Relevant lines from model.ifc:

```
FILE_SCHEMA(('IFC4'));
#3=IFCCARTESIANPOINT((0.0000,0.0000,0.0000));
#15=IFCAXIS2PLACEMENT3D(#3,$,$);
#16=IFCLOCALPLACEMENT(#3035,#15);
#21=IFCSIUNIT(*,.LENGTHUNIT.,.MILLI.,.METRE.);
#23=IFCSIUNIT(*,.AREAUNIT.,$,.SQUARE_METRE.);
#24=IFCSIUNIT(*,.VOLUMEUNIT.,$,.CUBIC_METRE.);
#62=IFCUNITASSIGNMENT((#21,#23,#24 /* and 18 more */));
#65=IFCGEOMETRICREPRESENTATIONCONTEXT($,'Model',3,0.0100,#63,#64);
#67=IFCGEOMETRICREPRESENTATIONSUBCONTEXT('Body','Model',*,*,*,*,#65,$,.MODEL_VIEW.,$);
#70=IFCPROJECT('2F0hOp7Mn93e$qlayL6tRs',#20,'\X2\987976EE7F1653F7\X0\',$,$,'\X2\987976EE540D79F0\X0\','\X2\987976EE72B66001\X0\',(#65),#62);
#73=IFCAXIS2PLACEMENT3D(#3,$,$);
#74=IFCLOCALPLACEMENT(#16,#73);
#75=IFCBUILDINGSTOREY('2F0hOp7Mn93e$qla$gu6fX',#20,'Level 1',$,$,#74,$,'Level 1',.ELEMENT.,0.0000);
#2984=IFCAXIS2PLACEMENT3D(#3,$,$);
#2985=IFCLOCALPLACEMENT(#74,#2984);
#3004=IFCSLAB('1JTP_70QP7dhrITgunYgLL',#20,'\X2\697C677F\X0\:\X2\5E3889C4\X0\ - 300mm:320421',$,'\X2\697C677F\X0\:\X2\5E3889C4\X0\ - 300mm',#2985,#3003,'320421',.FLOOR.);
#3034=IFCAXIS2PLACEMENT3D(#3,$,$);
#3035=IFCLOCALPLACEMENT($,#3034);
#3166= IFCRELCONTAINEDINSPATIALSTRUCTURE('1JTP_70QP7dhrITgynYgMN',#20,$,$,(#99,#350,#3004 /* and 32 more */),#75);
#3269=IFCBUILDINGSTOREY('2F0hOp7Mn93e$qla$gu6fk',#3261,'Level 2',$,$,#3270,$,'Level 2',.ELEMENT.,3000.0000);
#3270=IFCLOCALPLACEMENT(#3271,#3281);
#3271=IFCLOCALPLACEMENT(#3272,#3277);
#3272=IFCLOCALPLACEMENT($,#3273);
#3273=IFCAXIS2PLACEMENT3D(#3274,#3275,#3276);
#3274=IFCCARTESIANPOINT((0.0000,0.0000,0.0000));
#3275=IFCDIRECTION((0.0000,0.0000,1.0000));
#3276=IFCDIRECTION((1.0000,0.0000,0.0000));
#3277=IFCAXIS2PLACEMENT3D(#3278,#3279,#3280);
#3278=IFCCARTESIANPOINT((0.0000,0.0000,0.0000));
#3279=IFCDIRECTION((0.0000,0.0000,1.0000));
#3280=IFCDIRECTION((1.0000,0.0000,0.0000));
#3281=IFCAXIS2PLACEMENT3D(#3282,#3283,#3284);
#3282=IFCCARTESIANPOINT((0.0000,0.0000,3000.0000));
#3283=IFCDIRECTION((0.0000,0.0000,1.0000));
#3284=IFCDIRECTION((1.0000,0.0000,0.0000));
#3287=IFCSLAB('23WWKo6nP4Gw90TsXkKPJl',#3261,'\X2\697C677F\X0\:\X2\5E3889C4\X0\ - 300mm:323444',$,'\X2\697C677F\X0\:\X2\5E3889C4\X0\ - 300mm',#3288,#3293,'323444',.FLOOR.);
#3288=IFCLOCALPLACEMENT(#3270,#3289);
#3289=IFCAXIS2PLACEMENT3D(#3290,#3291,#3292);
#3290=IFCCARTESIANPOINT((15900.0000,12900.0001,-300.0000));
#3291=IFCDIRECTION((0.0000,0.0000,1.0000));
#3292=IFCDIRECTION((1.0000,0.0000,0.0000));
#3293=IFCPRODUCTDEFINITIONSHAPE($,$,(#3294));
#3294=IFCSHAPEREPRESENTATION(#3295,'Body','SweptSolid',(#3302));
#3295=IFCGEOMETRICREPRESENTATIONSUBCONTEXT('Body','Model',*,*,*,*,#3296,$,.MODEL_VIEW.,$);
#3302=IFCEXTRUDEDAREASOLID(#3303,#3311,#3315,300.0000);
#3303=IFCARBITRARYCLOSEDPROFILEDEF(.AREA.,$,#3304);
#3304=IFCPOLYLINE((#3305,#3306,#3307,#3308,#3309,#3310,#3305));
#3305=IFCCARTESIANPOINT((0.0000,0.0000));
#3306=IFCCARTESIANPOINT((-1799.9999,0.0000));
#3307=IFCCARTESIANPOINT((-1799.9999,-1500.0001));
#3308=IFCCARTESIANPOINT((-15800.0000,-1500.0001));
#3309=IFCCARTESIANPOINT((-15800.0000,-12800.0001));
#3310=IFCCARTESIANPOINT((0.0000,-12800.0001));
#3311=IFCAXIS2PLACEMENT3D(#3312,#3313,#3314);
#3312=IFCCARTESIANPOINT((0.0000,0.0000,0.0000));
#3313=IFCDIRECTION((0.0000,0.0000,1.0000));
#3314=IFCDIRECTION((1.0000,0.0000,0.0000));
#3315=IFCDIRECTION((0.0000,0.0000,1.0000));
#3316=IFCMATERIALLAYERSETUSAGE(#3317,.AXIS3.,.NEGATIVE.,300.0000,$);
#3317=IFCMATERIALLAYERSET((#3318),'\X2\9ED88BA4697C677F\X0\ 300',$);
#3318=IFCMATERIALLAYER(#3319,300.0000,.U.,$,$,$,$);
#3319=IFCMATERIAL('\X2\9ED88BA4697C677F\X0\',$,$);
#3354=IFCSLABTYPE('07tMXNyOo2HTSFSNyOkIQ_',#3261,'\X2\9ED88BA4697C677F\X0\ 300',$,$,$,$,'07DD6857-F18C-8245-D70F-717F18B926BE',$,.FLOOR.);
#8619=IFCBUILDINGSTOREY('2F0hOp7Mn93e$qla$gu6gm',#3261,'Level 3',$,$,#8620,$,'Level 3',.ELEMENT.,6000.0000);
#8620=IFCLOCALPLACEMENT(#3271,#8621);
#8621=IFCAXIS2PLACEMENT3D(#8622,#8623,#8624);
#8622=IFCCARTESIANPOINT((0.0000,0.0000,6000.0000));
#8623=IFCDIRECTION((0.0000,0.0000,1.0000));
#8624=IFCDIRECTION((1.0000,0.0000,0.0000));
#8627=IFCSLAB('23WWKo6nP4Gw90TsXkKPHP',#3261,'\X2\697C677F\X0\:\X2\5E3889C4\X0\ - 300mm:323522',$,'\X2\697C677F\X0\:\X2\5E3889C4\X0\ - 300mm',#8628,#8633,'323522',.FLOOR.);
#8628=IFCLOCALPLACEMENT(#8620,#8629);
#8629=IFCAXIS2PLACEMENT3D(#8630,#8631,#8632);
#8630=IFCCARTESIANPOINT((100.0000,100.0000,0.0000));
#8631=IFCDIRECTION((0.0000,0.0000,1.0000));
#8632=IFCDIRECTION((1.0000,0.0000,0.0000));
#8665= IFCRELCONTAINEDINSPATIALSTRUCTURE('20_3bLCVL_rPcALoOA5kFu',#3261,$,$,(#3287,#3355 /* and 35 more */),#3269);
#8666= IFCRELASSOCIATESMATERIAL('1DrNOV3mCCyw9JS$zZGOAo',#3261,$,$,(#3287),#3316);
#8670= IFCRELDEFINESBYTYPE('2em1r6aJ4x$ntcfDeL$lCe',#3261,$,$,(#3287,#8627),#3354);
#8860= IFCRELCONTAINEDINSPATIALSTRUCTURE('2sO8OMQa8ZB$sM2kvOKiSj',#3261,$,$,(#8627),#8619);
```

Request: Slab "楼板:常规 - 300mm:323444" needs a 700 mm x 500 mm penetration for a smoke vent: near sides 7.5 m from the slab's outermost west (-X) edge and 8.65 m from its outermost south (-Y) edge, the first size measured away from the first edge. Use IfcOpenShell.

```python
import numpy as np
import ifcopenshell
import ifcopenshell.api.feature
import ifcopenshell.api.geometry
import ifcopenshell.api.root
import ifcopenshell.geom
import ifcopenshell.util.placement
import ifcopenshell.util.representation
import ifcopenshell.util.shape
import ifcopenshell.util.unit

model = ifcopenshell.open("model.ifc")
unit_scale = ifcopenshell.util.unit.calculate_unit_scale(model)
settings = ifcopenshell.geom.settings()


def volume(element):
    """Net volume in cubic metres, openings subtracted."""
    shape = ifcopenshell.geom.create_shape(settings, element)
    return ifcopenshell.util.shape.get_volume(shape.geometry)


slab = model.by_id(3287)
before = volume(slab)

# Extent in the slab's own axes, in metres. The edges named are its -X and -Y sides.
slab_shape = ifcopenshell.geom.create_shape(settings, slab)
vertices = ifcopenshell.util.shape.get_vertices(slab_shape.geometry)
x_min, y_min, bottom = vertices.min(axis=0)
top = vertices[:, 2].max()

opening = ifcopenshell.api.root.create_entity(model, ifc_class="IfcOpeningElement", name="Smoke vent opening", predefined_type="OPENING")
context = ifcopenshell.util.representation.get_context(model, "Model", "Body", "MODEL_VIEW")
width, depth = 0.7, 0.5
outline = [(0.0, 0.0), (width, 0.0), (width, depth), (0.0, depth), (0.0, 0.0)]
# Overshoot both faces by 50 mm so the cut is clean.
shape = ifcopenshell.api.geometry.add_slab_representation(
    model, context=context, depth=top - bottom + 0.1, polyline=outline
)
ifcopenshell.api.geometry.assign_representation(model, product=opening, representation=shape)

matrix = ifcopenshell.util.placement.get_local_placement(slab.ObjectPlacement)
matrix[:, 3] = matrix @ np.append(np.array([x_min + 7.5, y_min + 8.65, bottom - 0.05]) / unit_scale, 1.0)
ifcopenshell.api.geometry.edit_object_placement(model, product=opening, matrix=matrix, is_si=False)
ifcopenshell.api.feature.add_feature(model, feature=opening, element=slab)

after = volume(slab)

print(f"slab volume {before:.3f} -> {after:.3f} m3")

model.write("model_rev.ifc")
```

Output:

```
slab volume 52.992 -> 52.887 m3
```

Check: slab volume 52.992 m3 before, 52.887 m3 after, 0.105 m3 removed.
